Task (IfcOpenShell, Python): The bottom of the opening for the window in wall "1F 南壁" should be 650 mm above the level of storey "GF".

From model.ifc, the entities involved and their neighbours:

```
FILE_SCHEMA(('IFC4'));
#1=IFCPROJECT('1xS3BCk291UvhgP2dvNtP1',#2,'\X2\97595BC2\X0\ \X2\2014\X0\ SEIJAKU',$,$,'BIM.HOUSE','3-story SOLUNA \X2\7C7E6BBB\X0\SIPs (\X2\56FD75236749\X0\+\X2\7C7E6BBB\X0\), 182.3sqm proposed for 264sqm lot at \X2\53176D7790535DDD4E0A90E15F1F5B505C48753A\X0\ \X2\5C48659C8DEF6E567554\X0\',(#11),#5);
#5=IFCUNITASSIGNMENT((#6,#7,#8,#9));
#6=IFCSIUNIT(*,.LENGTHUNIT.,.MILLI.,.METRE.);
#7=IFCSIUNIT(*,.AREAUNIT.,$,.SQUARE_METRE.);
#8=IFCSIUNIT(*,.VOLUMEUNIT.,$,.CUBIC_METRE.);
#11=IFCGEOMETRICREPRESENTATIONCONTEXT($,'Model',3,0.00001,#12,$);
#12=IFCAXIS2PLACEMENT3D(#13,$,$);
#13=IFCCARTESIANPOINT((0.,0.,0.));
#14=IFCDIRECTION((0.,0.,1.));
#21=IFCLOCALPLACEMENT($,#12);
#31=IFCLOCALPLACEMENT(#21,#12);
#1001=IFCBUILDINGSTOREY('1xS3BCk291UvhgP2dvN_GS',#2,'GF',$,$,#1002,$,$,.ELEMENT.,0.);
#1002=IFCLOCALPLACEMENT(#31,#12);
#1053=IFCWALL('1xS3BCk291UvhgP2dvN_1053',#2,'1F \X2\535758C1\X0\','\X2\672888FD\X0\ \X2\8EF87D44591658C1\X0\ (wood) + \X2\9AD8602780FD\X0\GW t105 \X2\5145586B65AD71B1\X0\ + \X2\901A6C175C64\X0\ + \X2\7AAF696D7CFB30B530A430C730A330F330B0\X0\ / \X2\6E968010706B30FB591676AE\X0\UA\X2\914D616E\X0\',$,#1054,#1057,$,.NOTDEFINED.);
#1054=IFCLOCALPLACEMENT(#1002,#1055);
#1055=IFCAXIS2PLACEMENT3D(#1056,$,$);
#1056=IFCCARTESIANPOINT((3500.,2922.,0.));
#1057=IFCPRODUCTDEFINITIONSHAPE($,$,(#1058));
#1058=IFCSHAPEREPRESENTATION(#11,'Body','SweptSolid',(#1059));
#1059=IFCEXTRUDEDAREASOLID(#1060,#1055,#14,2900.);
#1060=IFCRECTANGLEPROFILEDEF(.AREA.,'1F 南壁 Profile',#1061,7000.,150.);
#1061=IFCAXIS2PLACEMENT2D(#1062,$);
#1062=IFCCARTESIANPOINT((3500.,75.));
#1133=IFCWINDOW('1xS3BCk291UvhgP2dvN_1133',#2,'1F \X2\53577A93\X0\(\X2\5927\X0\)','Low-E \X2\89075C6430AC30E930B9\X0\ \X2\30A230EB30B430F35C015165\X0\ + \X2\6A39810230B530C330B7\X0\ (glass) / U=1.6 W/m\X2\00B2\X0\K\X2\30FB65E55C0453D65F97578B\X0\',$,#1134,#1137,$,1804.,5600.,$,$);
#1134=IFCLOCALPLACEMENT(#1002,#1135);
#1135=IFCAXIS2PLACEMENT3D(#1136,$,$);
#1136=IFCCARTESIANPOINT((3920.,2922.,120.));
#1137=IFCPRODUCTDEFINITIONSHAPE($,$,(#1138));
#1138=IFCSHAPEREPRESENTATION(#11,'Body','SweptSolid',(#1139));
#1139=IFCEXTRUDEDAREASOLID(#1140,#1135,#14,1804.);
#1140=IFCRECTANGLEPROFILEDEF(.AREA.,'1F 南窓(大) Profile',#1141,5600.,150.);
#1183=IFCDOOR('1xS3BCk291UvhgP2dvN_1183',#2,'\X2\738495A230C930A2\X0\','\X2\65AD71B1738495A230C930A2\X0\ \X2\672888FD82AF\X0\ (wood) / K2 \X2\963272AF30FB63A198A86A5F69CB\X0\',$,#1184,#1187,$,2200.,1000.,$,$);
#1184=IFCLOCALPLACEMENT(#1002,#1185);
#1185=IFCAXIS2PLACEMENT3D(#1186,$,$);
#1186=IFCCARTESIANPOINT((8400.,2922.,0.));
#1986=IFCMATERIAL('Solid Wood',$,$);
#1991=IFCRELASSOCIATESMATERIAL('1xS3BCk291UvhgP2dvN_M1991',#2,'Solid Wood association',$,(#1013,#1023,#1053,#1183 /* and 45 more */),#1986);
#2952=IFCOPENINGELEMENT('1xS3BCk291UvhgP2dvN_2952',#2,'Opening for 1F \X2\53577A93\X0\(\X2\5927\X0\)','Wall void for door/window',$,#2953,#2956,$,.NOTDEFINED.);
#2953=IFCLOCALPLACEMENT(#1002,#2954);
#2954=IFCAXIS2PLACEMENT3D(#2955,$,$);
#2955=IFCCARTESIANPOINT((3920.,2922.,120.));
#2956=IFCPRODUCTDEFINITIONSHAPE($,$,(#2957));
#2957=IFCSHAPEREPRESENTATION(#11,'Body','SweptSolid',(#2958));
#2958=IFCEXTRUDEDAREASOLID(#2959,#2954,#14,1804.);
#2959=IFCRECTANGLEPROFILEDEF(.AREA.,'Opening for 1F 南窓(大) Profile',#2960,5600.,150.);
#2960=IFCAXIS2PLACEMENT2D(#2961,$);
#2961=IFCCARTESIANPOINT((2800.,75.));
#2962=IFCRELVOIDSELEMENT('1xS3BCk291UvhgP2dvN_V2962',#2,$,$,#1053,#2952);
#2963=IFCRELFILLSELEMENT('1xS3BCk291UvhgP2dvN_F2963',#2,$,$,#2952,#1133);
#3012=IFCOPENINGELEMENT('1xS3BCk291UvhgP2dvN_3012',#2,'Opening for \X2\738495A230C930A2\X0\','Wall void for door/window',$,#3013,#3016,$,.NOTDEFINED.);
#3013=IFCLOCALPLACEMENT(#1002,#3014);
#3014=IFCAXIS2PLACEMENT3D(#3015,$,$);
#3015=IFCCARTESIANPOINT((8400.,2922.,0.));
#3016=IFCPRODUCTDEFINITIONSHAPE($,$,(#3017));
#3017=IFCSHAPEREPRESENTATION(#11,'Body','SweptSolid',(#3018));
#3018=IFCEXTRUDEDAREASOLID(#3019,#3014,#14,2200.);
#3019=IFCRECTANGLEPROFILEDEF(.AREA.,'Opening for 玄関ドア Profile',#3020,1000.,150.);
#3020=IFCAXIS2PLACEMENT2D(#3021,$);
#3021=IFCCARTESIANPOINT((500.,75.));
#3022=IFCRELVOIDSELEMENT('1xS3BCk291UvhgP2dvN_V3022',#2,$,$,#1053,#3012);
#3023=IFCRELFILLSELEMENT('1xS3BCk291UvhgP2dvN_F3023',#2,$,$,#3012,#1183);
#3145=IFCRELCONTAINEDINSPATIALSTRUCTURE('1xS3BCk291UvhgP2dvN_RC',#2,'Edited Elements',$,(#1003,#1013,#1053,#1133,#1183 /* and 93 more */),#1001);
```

```python
import numpy as np
import ifcopenshell
import ifcopenshell.api.geometry
import ifcopenshell.geom
import ifcopenshell.util.element
import ifcopenshell.util.placement
import ifcopenshell.util.shape
import ifcopenshell.util.unit

model = ifcopenshell.open("model.ifc")
unit_scale = ifcopenshell.util.unit.calculate_unit_scale(model)

window = model.by_id(1133)
opening = window.FillsVoids[0].RelatingOpeningElement
storey = ifcopenshell.util.element.get_container(window, ifc_class="IfcBuildingStorey")
level = ifcopenshell.util.placement.get_local_placement(storey.ObjectPlacement)[2, 3]

# The opening's origin need not be at the sill, so measure its lowest point.
shape = ifcopenshell.geom.create_shape(ifcopenshell.geom.settings(), opening)
bottom = ifcopenshell.util.shape.get_shape_bottom_elevation(shape, shape.geometry) / unit_scale
dz = level + 0.65 / unit_scale - bottom

shift = np.array([0.0, 0.0, dz])
# The window is not placed relative to its opening, so move both.
for product in (opening, window):
    matrix = ifcopenshell.util.placement.get_local_placement(product.ObjectPlacement)
    matrix[:3, 3] += shift
    ifcopenshell.api.geometry.edit_object_placement(model, product=product, matrix=matrix, is_si=False)

print(f"moved by {dz * unit_scale:+.3f} m")

model.write("model_edited.ifc")
```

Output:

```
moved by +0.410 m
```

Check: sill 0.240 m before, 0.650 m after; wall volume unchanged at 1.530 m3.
